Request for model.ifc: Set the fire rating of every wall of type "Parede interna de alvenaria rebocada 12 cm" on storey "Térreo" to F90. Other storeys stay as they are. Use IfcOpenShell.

First a look at what the model holds.

```python
import ifcopenshell
import ifcopenshell.util.element

model = ifcopenshell.open("model.ifc")
print(model.schema)
storey = next(s for s in model.by_type("IfcBuildingStorey") if s.Name == "Térreo")
walls = [e for e in ifcopenshell.util.element.get_decomposition(storey) if e.is_a("IfcWall")]
seen = {}
for e in walls:
    element_type = ifcopenshell.util.element.get_type(e)
    key = (element_type.Name if element_type != e and element_type else None, ifcopenshell.util.element.get_pset(e, "Pset_WallCommon", "FireRating"))
    seen[key] = seen.get(key, 0) + 1
for (name, value), count in sorted(seen.items(), key=str):
    print(count, "x", name, "|", value)
```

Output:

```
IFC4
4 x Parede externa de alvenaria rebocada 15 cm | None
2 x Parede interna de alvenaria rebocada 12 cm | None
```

```python
import ifcopenshell
import ifcopenshell.api.pset
import ifcopenshell.util.element

model = ifcopenshell.open("model.ifc")

storey = next(s for s in model.by_type("IfcBuildingStorey") if s.Name == "Térreo")
walls = [e for e in ifcopenshell.util.element.get_decomposition(storey) if e.is_a("IfcWall")]

count = 0
for e in walls:
    element_type = ifcopenshell.util.element.get_type(e)
    if element_type in (None, e) or element_type.Name != "Parede interna de alvenaria rebocada 12 cm":
        continue
    # add_pset returns the element's existing set when there is one.
    pset = ifcopenshell.api.pset.add_pset(model, product=e, name="Pset_WallCommon")
    ifcopenshell.api.pset.edit_pset(model, pset=pset, properties={"FireRating": "F90"})
    count += 1

print(count, "walls updated")

model.write("model_v2.ifc")
```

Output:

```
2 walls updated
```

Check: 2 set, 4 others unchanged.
